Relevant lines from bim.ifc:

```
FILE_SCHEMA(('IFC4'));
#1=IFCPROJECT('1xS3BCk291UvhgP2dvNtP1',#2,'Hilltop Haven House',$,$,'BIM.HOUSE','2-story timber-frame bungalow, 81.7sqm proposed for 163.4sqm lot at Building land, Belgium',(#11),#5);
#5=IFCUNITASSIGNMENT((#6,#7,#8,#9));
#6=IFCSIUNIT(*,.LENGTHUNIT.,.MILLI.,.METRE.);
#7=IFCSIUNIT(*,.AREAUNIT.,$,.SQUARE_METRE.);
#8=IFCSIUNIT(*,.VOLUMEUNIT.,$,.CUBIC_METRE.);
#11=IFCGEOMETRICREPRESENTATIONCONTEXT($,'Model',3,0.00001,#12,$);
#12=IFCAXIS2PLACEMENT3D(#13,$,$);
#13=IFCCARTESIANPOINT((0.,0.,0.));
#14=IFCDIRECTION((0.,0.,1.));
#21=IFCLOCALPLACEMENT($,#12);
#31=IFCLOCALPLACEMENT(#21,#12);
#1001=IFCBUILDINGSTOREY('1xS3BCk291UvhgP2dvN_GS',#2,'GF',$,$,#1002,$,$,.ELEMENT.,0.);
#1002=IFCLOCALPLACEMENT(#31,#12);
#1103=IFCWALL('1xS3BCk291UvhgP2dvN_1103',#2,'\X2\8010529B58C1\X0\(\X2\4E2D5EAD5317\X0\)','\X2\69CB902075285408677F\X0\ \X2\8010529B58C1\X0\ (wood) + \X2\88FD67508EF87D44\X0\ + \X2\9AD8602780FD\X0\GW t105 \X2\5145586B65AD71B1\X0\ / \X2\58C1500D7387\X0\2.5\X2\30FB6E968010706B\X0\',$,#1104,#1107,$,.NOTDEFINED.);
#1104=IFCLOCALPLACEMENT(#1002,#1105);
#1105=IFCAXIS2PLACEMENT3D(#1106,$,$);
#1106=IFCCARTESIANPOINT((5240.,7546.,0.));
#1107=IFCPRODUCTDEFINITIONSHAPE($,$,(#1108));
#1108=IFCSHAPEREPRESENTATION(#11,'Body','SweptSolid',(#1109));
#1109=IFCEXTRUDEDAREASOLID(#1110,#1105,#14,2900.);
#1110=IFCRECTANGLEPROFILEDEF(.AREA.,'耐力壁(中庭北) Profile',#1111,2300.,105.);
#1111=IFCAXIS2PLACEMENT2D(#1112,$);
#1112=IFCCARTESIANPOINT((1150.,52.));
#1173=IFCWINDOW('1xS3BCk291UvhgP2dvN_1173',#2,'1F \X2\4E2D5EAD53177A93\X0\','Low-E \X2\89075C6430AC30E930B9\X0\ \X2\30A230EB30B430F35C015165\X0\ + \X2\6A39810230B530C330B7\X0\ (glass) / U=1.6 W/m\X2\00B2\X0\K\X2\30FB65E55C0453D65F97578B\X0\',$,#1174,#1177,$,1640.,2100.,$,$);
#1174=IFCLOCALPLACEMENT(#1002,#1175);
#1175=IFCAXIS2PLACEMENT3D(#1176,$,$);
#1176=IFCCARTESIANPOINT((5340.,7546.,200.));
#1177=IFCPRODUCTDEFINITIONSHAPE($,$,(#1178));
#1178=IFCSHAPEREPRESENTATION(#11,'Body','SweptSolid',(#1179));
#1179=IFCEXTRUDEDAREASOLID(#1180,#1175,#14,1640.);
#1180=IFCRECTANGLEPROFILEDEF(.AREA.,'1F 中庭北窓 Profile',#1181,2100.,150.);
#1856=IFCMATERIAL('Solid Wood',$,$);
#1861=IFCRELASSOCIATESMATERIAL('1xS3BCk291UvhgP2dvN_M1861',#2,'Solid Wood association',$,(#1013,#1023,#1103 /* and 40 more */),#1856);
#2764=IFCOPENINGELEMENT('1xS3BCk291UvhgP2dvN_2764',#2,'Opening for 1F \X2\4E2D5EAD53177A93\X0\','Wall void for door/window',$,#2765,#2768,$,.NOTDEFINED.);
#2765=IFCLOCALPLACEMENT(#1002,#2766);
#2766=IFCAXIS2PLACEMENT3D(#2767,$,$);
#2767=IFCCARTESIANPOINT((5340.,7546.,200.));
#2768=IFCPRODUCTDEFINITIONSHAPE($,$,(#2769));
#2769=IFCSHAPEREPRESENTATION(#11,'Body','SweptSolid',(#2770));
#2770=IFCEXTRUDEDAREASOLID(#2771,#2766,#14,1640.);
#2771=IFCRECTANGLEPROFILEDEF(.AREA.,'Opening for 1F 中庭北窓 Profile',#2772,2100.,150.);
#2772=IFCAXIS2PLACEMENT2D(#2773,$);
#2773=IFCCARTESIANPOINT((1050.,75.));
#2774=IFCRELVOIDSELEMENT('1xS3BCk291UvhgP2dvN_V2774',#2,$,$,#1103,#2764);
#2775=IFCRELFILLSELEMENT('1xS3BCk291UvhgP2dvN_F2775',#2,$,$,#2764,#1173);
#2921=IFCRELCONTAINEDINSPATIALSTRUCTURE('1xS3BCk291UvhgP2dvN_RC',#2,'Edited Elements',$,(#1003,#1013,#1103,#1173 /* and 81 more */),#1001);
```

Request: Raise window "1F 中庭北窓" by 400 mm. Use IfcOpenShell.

```python
import numpy as np
import ifcopenshell
import ifcopenshell.api.geometry
import ifcopenshell.util.placement
import ifcopenshell.util.unit

model = ifcopenshell.open("bim.ifc")
unit_scale = ifcopenshell.util.unit.calculate_unit_scale(model)

window = model.by_guid("1xS3BCk291UvhgP2dvN_1173")
opening = window.FillsVoids[0].RelatingOpeningElement
dz = 0.4 / unit_scale

shift = np.array([0.0, 0.0, dz])
# The window is not placed relative to its opening, so move both.
for product in (opening, window):
    matrix = ifcopenshell.util.placement.get_local_placement(product.ObjectPlacement)
    matrix[:3, 3] += shift
    ifcopenshell.api.geometry.edit_object_placement(model, product=product, matrix=matrix, is_si=False)

print(f"moved by {dz * unit_scale:+.3f} m")

model.write("bim_updated.ifc")
```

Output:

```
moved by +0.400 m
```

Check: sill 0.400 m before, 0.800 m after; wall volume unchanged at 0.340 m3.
